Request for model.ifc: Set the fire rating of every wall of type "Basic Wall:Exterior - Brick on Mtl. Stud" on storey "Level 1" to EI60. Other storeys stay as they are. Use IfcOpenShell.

First a look at what the model holds.

```python
import ifcopenshell
import ifcopenshell.util.element

model = ifcopenshell.open("model.ifc")
print(model.schema)
storey = next(s for s in model.by_type("IfcBuildingStorey") if s.Name == "Level 1")
walls = [e for e in ifcopenshell.util.element.get_decomposition(storey) if e.is_a("IfcWall")]
seen = {}
for e in walls:
    element_type = ifcopenshell.util.element.get_type(e)
    key = (element_type.Name if element_type != e and element_type else None, ifcopenshell.util.element.get_pset(e, "Pset_WallCommon", "FireRating"))
    seen[key] = seen.get(key, 0) + 1
for (name, value), count in sorted(seen.items(), key=str):
    print(count, "x", name, "|", value)
```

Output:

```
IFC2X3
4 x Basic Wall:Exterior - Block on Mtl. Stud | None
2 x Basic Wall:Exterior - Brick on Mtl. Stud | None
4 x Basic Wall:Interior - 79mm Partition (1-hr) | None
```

```python
import ifcopenshell
import ifcopenshell.api.pset
import ifcopenshell.util.element

model = ifcopenshell.open("model.ifc")

storey = next(s for s in model.by_type("IfcBuildingStorey") if s.Name == "Level 1")
walls = [e for e in ifcopenshell.util.element.get_decomposition(storey) if e.is_a("IfcWall")]

count = 0
for e in walls:
    element_type = ifcopenshell.util.element.get_type(e)
    if element_type in (None, e) or element_type.Name != "Basic Wall:Exterior - Brick on Mtl. Stud":
        continue
    # add_pset returns the element's existing set when there is one.
    pset = ifcopenshell.api.pset.add_pset(model, product=e, name="Pset_WallCommon")
    ifcopenshell.api.pset.edit_pset(model, pset=pset, properties={"FireRating": "EI60"})
    count += 1

print(count, "walls updated")

model.write("model-out.ifc")
```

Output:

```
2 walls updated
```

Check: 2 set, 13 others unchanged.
